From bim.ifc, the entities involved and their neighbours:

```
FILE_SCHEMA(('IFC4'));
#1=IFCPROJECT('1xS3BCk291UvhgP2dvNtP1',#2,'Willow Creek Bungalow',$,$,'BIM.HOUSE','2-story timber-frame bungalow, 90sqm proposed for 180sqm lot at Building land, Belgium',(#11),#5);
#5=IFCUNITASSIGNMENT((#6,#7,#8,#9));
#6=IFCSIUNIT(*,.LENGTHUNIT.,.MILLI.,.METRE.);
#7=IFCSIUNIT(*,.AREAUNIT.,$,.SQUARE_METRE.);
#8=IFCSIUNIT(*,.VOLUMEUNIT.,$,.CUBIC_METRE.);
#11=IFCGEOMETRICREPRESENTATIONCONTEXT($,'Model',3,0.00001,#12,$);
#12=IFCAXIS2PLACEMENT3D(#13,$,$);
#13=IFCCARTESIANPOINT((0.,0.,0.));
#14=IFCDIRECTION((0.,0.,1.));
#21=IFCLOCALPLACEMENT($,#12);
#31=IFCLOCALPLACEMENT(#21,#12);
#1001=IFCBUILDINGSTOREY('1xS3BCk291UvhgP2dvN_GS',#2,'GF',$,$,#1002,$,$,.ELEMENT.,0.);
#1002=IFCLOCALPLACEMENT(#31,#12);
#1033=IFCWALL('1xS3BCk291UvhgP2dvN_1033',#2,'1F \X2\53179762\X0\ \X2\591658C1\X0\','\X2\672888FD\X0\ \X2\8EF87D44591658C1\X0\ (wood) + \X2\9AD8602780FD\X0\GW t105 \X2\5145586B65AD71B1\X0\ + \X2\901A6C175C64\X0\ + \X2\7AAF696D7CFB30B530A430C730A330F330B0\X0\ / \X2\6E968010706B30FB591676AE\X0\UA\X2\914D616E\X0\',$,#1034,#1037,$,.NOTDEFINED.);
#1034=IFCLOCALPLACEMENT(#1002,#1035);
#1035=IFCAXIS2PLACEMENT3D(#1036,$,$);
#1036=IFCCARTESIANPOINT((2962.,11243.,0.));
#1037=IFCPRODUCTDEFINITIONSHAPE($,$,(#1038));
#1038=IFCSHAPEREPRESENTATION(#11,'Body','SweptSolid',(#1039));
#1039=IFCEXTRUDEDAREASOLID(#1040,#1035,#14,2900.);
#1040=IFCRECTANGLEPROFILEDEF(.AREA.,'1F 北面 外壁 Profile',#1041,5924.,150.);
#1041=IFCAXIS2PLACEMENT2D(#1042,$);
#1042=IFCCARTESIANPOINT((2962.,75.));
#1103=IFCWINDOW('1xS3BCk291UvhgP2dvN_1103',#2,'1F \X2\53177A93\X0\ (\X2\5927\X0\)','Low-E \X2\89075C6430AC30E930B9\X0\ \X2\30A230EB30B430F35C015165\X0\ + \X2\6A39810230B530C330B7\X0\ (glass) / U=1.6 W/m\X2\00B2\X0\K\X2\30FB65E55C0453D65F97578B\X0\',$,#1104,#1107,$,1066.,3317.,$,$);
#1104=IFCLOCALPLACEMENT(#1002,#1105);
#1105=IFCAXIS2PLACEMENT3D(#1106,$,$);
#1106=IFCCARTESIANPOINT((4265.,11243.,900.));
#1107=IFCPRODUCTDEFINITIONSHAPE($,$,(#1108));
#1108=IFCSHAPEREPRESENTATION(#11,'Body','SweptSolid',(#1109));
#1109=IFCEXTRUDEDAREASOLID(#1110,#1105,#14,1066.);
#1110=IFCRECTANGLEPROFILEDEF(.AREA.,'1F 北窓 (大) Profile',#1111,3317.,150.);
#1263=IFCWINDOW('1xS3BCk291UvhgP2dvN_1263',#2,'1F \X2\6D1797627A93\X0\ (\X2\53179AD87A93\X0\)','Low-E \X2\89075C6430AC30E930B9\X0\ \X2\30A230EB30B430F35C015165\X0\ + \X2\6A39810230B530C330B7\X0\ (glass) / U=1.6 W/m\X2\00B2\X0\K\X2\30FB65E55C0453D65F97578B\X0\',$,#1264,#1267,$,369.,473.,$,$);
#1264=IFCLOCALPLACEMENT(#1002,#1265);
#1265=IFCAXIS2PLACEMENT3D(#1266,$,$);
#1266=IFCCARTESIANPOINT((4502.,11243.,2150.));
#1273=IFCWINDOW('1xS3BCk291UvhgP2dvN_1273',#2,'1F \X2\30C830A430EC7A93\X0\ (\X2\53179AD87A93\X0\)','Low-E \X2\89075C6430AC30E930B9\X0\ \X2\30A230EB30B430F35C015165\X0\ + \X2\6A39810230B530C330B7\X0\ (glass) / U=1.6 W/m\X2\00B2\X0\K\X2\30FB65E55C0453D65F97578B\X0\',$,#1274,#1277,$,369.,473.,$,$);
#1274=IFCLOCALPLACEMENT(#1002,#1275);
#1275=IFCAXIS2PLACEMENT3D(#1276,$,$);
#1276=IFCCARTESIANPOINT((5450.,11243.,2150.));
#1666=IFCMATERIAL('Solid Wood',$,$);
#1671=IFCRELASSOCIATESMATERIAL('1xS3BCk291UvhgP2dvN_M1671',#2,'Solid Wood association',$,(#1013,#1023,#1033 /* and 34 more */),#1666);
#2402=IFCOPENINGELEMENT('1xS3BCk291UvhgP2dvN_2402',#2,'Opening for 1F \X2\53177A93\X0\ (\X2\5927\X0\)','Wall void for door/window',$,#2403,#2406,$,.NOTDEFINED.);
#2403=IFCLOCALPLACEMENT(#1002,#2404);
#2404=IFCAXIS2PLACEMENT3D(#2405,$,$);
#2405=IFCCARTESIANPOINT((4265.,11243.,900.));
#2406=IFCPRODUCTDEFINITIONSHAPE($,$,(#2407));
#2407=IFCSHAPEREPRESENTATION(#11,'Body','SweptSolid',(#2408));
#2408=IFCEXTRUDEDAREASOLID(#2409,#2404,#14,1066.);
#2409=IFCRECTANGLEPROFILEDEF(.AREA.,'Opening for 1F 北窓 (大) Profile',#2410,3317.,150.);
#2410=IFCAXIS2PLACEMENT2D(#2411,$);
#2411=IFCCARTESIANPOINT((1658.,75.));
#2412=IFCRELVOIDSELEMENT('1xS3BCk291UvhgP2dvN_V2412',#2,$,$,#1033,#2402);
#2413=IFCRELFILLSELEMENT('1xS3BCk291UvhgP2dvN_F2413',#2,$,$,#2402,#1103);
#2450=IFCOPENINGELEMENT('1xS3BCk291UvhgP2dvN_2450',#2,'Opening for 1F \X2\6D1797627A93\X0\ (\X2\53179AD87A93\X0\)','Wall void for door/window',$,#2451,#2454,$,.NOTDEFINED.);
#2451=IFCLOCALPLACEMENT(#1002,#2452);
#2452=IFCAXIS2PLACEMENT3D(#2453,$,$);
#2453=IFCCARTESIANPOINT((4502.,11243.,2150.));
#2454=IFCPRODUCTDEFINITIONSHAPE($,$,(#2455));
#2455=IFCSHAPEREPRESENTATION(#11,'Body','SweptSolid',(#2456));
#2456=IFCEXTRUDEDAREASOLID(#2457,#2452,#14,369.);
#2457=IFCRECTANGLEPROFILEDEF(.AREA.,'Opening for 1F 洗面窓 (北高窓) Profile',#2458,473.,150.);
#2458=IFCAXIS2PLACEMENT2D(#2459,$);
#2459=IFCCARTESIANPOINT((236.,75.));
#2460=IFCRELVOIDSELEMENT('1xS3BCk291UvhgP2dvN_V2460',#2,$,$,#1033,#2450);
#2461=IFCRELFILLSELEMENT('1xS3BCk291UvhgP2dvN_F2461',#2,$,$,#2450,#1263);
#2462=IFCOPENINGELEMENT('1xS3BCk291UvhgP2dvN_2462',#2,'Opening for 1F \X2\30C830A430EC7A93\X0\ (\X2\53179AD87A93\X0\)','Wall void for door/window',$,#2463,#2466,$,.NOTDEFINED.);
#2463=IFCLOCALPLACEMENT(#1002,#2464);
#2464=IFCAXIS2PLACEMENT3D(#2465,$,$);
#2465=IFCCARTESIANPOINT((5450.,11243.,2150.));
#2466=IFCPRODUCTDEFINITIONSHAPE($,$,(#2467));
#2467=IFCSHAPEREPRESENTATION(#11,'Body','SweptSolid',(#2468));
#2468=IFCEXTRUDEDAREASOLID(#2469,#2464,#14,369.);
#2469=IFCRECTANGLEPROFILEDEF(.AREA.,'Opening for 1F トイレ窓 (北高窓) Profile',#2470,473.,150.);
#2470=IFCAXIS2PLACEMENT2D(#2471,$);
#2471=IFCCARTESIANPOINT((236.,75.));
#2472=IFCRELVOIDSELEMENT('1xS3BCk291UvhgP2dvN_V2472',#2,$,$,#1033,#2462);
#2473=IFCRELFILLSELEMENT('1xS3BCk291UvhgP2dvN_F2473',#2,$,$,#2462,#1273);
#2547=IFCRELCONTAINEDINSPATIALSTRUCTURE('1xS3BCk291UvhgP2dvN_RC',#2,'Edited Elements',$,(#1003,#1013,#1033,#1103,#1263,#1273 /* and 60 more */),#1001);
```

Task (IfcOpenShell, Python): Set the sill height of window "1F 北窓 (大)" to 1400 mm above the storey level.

```python
import numpy as np
import ifcopenshell
import ifcopenshell.api.geometry
import ifcopenshell.geom
import ifcopenshell.util.element
import ifcopenshell.util.placement
import ifcopenshell.util.shape
import ifcopenshell.util.unit

model = ifcopenshell.open("bim.ifc")
unit_scale = ifcopenshell.util.unit.calculate_unit_scale(model)

window = model.by_id(1103)
opening = window.FillsVoids[0].RelatingOpeningElement
storey = ifcopenshell.util.element.get_container(window, ifc_class="IfcBuildingStorey")
level = ifcopenshell.util.placement.get_local_placement(storey.ObjectPlacement)[2, 3]

# The opening's origin need not be at the sill, so measure its lowest point.
shape = ifcopenshell.geom.create_shape(ifcopenshell.geom.settings(), opening)
bottom = ifcopenshell.util.shape.get_shape_bottom_elevation(shape, shape.geometry) / unit_scale
dz = level + 1400.0 - bottom

shift = np.array([0.0, 0.0, dz])
# The window is not placed relative to its opening, so move both.
for product in (opening, window):
    matrix = ifcopenshell.util.placement.get_local_placement(product.ObjectPlacement)
    matrix[:3, 3] += shift
    ifcopenshell.api.geometry.edit_object_placement(model, product=product, matrix=matrix, is_si=False)

print(f"moved by {dz * unit_scale:+.3f} m")

model.write("bim_edited.ifc")
```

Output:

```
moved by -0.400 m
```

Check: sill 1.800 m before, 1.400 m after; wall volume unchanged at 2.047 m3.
